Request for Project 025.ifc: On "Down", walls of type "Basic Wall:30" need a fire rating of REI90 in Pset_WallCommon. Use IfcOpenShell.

First a look at what the model holds.

```python
import ifcopenshell
import ifcopenshell.util.element

model = ifcopenshell.open("Project 025.ifc")
print(model.schema)
storey = next(s for s in model.by_type("IfcBuildingStorey") if s.Name == "Down")
walls = [e for e in ifcopenshell.util.element.get_decomposition(storey) if e.is_a("IfcWall")]
seen = {}
for e in walls:
    element_type = ifcopenshell.util.element.get_type(e)
    key = (element_type.Name if element_type != e and element_type else None, ifcopenshell.util.element.get_pset(e, "Pset_WallCommon", "FireRating"))
    seen[key] = seen.get(key, 0) + 1
for (name, value), count in sorted(seen.items(), key=str):
    print(count, "x", name, "|", value)
```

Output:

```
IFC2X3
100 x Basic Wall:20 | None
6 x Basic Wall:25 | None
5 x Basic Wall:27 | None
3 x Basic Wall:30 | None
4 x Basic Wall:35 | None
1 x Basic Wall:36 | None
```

```python
import ifcopenshell
import ifcopenshell.api.pset
import ifcopenshell.util.element

model = ifcopenshell.open("Project 025.ifc")

storey = next(s for s in model.by_type("IfcBuildingStorey") if s.Name == "Down")
walls = [e for e in ifcopenshell.util.element.get_decomposition(storey) if e.is_a("IfcWall")]

count = 0
for e in walls:
    element_type = ifcopenshell.util.element.get_type(e)
    if element_type in (None, e) or element_type.Name != "Basic Wall:30":
        continue
    # add_pset returns the element's existing set when there is one.
    pset = ifcopenshell.api.pset.add_pset(model, product=e, name="Pset_WallCommon")
    ifcopenshell.api.pset.edit_pset(model, pset=pset, properties={"FireRating": "REI90"})
    count += 1

print(count, "walls updated")

model.write("Project 025_v2.ifc")
```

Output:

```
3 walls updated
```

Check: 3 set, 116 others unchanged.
